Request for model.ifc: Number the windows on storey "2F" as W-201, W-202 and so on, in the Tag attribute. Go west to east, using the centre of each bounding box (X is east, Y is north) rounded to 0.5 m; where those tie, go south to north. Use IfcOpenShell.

First a look at what the model holds.

```python
import ifcopenshell
import ifcopenshell.util.element
import ifcopenshell.util.placement

model = ifcopenshell.open("model.ifc")
print(model.schema)
storey = next(s for s in model.by_type("IfcBuildingStorey") if s.Name == "2F")
windows = [e for e in ifcopenshell.util.element.get_decomposition(storey) if e.is_a("IfcWindow")]
for e in sorted(windows, key=lambda e: e.id()):
    origin = ifcopenshell.util.placement.get_local_placement(e.ObjectPlacement)[:3, 3]
    print(e.id(), e.Tag, e.Name, origin.round(2) + 0.0, sep=" | ")
```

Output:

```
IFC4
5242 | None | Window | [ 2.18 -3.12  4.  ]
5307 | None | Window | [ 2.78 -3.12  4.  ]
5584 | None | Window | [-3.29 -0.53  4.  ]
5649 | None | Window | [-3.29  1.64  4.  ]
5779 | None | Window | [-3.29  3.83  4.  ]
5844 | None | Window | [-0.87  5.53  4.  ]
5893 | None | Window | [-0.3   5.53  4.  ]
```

```python
import ifcopenshell
import ifcopenshell.geom
import ifcopenshell.util.element
import ifcopenshell.util.shape

model = ifcopenshell.open("model.ifc")
settings = ifcopenshell.geom.settings()
settings.set("use-world-coords", True)


def centre(element):
    shape = ifcopenshell.geom.create_shape(settings, element)
    return ifcopenshell.util.shape.get_bbox_centroid(shape.geometry)


storey = next(s for s in model.by_type("IfcBuildingStorey") if s.Name == "2F")
windows = [e for e in ifcopenshell.util.element.get_decomposition(storey) if e.is_a("IfcWindow")]

# Insertion points can sit at a corner or the storey origin, so sort by the geometry (in metres).
centres = {e: centre(e) for e in windows}
windows.sort(key=lambda e: (round(centres[e][0] / 0.5), centres[e][1]))

for i, e in enumerate(windows, start=1):
    number = f"W-2{i:02d}"
    e.Tag = number
    print(e.id(), number)

model.write("model-out.ifc")
```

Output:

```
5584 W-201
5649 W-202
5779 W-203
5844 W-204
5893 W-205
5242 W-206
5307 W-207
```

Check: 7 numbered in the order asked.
